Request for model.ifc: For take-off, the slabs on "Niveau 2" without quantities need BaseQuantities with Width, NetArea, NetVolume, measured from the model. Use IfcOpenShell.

First a look at what the model holds.

```python
import ifcopenshell
import ifcopenshell.util.element
import ifcopenshell.util.unit

model = ifcopenshell.open("model.ifc")
print(model.schema)
for unit_type in ("LENGTHUNIT", "AREAUNIT", "VOLUMEUNIT"):
    print(unit_type, ifcopenshell.util.unit.calculate_unit_scale(model, unit_type))
storey = next(s for s in model.by_type("IfcBuildingStorey") if s.Name == "Niveau 2")
slabs = [e for e in ifcopenshell.util.element.get_decomposition(storey) if e.is_a("IfcSlab")]
for e in sorted(slabs, key=lambda e: e.id()):
    print(e.id(), e.is_a(), e.Name, list(ifcopenshell.util.element.get_psets(e, qtos_only=True)), sep=" | ")
```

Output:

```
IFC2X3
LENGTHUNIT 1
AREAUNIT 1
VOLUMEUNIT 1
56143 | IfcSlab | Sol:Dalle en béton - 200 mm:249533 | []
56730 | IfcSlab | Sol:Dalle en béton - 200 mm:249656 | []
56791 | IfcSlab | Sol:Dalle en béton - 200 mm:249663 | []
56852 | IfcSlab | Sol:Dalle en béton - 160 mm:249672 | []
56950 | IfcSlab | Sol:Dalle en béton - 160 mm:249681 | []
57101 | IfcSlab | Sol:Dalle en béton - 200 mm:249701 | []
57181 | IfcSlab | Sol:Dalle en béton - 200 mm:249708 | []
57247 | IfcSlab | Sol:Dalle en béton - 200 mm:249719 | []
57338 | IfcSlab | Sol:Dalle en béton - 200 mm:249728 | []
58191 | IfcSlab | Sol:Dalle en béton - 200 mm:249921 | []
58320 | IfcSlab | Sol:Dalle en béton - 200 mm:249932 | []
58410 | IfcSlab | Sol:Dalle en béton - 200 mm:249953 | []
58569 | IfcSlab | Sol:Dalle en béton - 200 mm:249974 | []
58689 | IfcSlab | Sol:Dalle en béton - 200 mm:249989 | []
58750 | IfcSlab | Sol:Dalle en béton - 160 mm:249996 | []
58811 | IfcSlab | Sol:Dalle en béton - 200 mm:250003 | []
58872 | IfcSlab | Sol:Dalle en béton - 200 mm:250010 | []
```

```python
import ifcopenshell
import ifcopenshell.api.pset
import ifcopenshell.geom
import ifcopenshell.util.element
import ifcopenshell.util.shape
import ifcopenshell.util.unit

model = ifcopenshell.open("model.ifc")
unit_scale = ifcopenshell.util.unit.calculate_unit_scale(model)
area_scale = ifcopenshell.util.unit.calculate_unit_scale(model, "AREAUNIT")
volume_scale = ifcopenshell.util.unit.calculate_unit_scale(model, "VOLUMEUNIT")
settings = ifcopenshell.geom.settings()

storey = next(s for s in model.by_type("IfcBuildingStorey") if s.Name == "Niveau 2")
slabs = [e for e in ifcopenshell.util.element.get_decomposition(storey) if e.is_a("IfcSlab")]

for e in sorted(slabs, key=lambda e: e.id()):
    if ifcopenshell.util.element.get_psets(e, qtos_only=True, should_inherit=False):
        continue
    # Geometry comes back in metres, in the element's own axes.
    shape = ifcopenshell.geom.create_shape(settings, e)
    values = {
        "Width": ifcopenshell.util.shape.get_z(shape.geometry) / unit_scale,
        "NetArea": ifcopenshell.util.shape.get_footprint_area(shape.geometry) / area_scale,
        "NetVolume": ifcopenshell.util.shape.get_volume(shape.geometry) / volume_scale,
    }
    qto = ifcopenshell.api.pset.add_qto(model, product=e, name="BaseQuantities")
    ifcopenshell.api.pset.edit_qto(model, qto=qto, properties=values)
    print(e.id(), {k: round(v, 3) for k, v in values.items()})

model.write("model_updated.ifc")
```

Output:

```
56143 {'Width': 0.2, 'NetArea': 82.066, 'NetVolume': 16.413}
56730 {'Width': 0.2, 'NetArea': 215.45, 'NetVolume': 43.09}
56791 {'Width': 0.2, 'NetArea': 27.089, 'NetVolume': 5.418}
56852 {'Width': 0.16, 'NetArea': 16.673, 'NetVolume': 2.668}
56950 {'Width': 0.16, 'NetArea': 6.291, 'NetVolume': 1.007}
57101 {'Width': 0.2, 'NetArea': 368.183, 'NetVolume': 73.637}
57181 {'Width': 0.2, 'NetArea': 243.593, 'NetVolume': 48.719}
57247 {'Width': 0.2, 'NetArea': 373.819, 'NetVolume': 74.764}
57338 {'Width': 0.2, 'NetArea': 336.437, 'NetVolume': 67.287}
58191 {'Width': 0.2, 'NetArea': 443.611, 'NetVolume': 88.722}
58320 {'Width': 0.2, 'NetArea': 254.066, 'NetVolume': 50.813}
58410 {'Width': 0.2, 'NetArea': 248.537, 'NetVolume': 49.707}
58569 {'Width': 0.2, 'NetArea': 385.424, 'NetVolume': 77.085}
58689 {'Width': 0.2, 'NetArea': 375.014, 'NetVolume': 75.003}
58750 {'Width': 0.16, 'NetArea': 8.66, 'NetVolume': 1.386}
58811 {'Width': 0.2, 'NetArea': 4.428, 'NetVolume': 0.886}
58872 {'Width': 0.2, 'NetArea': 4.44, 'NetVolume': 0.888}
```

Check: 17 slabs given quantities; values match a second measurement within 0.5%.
